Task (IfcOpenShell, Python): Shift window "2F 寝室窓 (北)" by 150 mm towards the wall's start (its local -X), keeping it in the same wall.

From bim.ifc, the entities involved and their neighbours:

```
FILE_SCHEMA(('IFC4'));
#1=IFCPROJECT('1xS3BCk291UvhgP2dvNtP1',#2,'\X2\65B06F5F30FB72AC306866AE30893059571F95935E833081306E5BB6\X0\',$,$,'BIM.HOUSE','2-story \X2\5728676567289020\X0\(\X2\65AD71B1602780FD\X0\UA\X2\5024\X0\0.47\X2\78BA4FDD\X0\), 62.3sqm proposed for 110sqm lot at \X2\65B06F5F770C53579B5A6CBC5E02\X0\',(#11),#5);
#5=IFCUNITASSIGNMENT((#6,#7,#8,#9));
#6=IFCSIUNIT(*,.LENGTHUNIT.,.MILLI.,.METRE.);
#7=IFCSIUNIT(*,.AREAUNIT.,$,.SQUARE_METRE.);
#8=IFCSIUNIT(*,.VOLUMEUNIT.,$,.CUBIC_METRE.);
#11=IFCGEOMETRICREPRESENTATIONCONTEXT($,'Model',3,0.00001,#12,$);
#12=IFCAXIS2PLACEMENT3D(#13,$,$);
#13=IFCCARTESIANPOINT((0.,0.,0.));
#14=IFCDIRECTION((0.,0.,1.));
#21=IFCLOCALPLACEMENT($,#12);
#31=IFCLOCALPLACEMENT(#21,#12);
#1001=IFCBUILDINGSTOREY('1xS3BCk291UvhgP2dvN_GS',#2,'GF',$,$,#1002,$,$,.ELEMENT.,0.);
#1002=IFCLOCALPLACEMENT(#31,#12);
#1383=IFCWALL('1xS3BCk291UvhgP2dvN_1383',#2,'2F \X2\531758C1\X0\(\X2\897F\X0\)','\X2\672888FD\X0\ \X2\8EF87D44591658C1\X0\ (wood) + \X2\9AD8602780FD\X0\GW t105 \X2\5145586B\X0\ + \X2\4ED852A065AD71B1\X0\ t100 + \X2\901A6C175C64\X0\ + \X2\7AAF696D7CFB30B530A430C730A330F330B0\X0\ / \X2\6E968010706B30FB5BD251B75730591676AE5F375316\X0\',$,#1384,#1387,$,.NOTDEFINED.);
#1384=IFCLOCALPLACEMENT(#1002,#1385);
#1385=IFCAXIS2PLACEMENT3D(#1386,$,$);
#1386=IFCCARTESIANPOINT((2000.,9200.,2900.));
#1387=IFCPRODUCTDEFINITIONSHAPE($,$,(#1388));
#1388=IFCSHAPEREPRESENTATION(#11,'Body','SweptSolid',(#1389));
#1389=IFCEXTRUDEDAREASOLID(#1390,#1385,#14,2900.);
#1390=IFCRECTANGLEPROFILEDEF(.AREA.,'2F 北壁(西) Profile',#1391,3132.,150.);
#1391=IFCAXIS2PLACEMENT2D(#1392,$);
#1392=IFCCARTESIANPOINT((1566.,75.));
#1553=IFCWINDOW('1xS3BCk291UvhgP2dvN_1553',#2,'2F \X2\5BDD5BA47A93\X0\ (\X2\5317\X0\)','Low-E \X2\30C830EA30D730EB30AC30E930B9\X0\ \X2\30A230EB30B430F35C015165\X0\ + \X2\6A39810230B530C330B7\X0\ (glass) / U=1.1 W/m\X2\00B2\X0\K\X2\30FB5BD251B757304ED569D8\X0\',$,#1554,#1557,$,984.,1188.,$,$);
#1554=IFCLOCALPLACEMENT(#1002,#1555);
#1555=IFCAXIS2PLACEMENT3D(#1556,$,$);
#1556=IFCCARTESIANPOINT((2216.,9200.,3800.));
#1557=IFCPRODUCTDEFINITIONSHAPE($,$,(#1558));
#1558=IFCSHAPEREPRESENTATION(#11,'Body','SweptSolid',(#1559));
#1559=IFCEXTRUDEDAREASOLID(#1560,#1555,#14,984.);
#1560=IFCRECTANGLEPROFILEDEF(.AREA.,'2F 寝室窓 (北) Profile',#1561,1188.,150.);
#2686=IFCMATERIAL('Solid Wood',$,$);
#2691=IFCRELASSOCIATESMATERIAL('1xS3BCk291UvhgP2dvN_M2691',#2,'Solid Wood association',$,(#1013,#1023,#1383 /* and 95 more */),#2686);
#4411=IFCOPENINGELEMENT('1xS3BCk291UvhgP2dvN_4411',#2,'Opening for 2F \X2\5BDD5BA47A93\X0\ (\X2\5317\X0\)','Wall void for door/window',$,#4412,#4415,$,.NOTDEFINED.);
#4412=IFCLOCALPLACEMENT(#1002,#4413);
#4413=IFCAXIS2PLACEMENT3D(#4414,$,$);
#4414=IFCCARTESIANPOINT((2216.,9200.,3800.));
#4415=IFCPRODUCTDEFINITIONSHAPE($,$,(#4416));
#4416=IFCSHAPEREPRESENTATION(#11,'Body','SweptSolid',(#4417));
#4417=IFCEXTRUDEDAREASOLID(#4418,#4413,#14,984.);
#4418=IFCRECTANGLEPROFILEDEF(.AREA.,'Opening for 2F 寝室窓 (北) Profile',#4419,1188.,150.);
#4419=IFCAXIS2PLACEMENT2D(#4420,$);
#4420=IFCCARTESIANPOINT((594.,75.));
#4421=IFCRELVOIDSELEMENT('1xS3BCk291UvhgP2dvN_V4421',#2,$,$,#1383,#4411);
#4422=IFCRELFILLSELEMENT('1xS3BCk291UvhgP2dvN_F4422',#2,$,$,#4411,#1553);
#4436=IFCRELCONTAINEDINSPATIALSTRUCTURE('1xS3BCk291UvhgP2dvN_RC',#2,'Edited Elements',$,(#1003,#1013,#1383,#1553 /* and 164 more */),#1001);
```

```python
import ifcopenshell
import ifcopenshell.api.geometry
import ifcopenshell.util.placement
import ifcopenshell.util.unit

model = ifcopenshell.open("bim.ifc")
unit_scale = ifcopenshell.util.unit.calculate_unit_scale(model)

window = model.by_guid("1xS3BCk291UvhgP2dvN_1553")
opening = window.FillsVoids[0].RelatingOpeningElement
wall = opening.VoidsElements[0].RelatingBuildingElement

wall_matrix = ifcopenshell.util.placement.get_local_placement(wall.ObjectPlacement)
shift = wall_matrix[:3, 0] * -0.15 / unit_scale
before = ifcopenshell.util.placement.get_local_placement(window.ObjectPlacement)[:3, 3].copy()

# The window is not placed relative to its opening, so move both.
for product in (opening, window):
    matrix = ifcopenshell.util.placement.get_local_placement(product.ObjectPlacement)
    matrix[:3, 3] += shift
    ifcopenshell.api.geometry.edit_object_placement(model, product=product, matrix=matrix, is_si=False)

after = ifcopenshell.util.placement.get_local_placement(window.ObjectPlacement)[:3, 3]
print("window moved by", (after - before).round(3) + 0.0)

model.write("bim_rev.ifc")
```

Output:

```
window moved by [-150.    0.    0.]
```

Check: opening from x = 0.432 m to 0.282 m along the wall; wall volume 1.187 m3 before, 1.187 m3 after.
